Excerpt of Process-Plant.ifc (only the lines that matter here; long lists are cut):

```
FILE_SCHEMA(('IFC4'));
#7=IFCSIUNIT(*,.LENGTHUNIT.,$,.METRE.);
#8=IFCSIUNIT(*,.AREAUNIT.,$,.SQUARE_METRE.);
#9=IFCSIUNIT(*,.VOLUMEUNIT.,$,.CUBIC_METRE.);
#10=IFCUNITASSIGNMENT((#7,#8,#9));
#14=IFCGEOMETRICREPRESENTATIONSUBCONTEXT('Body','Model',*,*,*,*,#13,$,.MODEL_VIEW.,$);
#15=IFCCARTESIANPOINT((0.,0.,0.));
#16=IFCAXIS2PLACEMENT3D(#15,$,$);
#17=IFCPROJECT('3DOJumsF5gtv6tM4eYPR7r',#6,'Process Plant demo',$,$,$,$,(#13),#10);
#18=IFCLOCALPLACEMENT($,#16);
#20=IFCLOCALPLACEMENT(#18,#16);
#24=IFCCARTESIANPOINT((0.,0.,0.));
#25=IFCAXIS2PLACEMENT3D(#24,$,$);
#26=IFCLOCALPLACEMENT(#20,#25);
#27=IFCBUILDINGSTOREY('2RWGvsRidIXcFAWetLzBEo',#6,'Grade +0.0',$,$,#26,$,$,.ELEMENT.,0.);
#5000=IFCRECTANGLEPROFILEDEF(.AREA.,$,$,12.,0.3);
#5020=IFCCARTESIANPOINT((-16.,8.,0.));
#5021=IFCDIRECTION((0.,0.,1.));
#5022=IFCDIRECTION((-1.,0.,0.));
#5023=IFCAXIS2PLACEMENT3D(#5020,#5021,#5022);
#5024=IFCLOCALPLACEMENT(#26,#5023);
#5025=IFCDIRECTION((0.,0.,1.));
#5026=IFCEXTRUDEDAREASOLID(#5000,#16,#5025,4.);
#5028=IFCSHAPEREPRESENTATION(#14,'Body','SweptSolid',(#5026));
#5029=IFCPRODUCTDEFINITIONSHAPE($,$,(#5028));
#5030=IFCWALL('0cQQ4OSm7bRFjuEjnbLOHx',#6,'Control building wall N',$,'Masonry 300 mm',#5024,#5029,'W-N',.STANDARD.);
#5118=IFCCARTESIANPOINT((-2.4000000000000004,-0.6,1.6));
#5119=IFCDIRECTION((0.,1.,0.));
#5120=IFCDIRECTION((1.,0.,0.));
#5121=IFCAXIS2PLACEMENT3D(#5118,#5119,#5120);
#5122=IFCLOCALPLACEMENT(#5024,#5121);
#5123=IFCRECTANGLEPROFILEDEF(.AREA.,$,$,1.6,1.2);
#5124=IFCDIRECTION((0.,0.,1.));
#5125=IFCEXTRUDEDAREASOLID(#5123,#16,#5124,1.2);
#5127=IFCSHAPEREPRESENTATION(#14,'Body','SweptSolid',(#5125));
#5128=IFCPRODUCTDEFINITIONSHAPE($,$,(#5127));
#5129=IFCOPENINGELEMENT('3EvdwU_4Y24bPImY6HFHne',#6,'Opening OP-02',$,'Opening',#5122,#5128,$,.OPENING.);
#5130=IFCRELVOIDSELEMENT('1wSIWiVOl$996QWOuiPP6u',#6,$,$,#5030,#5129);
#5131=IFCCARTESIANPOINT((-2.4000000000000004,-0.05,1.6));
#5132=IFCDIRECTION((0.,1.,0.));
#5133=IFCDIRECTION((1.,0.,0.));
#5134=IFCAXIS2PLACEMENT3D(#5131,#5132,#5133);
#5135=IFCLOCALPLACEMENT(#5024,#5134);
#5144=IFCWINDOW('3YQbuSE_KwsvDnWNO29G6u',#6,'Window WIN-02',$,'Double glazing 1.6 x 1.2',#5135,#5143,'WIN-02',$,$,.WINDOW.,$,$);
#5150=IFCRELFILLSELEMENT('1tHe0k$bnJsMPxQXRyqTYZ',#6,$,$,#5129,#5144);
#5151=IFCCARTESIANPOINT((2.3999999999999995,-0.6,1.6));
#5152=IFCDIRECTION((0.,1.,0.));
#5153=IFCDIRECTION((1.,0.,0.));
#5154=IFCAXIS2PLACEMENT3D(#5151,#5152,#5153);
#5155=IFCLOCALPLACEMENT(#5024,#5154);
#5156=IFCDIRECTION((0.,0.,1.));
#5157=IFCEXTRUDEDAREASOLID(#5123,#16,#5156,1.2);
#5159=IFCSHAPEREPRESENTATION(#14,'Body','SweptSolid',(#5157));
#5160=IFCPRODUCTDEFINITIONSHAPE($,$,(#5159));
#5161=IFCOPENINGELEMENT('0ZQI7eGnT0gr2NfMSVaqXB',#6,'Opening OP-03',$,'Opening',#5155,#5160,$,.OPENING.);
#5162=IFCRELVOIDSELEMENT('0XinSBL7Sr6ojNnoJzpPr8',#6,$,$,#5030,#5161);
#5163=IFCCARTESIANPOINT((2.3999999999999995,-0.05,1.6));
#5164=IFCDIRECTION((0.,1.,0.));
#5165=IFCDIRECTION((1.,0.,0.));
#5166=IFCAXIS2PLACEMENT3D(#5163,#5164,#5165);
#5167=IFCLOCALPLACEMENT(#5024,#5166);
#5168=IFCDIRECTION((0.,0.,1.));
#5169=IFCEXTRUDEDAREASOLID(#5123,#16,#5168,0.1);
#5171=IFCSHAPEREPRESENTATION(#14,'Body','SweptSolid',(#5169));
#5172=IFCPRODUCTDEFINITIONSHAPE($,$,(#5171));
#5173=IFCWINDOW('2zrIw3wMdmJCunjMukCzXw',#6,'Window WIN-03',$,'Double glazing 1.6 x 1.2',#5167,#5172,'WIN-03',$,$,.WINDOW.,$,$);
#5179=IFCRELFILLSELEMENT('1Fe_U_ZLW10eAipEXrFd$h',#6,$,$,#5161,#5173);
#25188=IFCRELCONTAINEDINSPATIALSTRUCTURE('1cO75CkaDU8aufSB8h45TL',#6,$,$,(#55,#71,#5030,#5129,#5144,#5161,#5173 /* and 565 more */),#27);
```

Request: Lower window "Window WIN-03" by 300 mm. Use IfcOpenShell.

```python
import numpy as np
import ifcopenshell
import ifcopenshell.api.geometry
import ifcopenshell.util.placement
import ifcopenshell.util.unit

model = ifcopenshell.open("Process-Plant.ifc")
unit_scale = ifcopenshell.util.unit.calculate_unit_scale(model)

window = model.by_guid("2zrIw3wMdmJCunjMukCzXw")
opening = window.FillsVoids[0].RelatingOpeningElement
dz = -0.3

shift = np.array([0.0, 0.0, dz])
# The window is not placed relative to its opening, so move both.
for product in (opening, window):
    matrix = ifcopenshell.util.placement.get_local_placement(product.ObjectPlacement)
    matrix[:3, 3] += shift
    ifcopenshell.api.geometry.edit_object_placement(model, product=product, matrix=matrix, is_si=False)

print(f"moved by {dz * unit_scale:+.3f} m")

model.write("Process-Plant_edited.ifc")
```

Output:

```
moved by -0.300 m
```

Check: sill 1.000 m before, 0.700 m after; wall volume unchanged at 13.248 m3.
